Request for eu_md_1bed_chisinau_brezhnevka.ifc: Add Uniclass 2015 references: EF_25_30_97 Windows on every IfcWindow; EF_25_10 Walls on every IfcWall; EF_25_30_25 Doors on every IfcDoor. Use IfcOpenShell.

First a look at what the model holds.

```python
import ifcopenshell

model = ifcopenshell.open("eu_md_1bed_chisinau_brezhnevka.ifc")
print(model.schema)
print("classifications:", [c.Name for c in model.by_type("IfcClassification")])
for ifc_class in ("IfcDoor", "IfcRoof", "IfcStair", "IfcWall", "IfcWindow"):
    print(ifc_class, len(model.by_type(ifc_class)))
```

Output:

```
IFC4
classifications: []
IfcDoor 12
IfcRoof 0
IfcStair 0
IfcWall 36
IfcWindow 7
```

```python
import ifcopenshell
import ifcopenshell.api.classification

model = ifcopenshell.open("eu_md_1bed_chisinau_brezhnevka.ifc")

system = ifcopenshell.api.classification.add_classification(model, classification="Uniclass 2015")

codes = {
    "IfcWindow": ("EF_25_30_97", "Windows"),
    "IfcWall": ("EF_25_10", "Walls"),
    "IfcDoor": ("EF_25_30_25", "Doors"),
}
for ifc_class, (code, name) in codes.items():
    products = model.by_type(ifc_class)
    ifcopenshell.api.classification.add_reference(
        model, products=products, classification=system, identification=code, name=name
    )
    print(code, len(products))

model.write("eu_md_1bed_chisinau_brezhnevka_updated.ifc")
```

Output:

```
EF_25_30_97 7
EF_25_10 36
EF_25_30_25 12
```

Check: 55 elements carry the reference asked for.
